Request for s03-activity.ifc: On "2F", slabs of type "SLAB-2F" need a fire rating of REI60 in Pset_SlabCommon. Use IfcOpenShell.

First a look at what the model holds.

```python
import ifcopenshell
import ifcopenshell.util.element

model = ifcopenshell.open("s03-activity.ifc")
print(model.schema)
storey = next(s for s in model.by_type("IfcBuildingStorey") if s.Name == "2F")
slabs = [e for e in ifcopenshell.util.element.get_decomposition(storey) if e.is_a("IfcSlab")]
seen = {}
for e in slabs:
    element_type = ifcopenshell.util.element.get_type(e)
    key = (element_type.Name if element_type != e and element_type else None, ifcopenshell.util.element.get_pset(e, "Pset_SlabCommon", "FireRating"))
    seen[key] = seen.get(key, 0) + 1
for (name, value), count in sorted(seen.items(), key=str):
    print(count, "x", name, "|", value)
```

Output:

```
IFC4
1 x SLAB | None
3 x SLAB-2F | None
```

```python
import ifcopenshell
import ifcopenshell.api.pset
import ifcopenshell.util.element

model = ifcopenshell.open("s03-activity.ifc")

storey = next(s for s in model.by_type("IfcBuildingStorey") if s.Name == "2F")
slabs = [e for e in ifcopenshell.util.element.get_decomposition(storey) if e.is_a("IfcSlab")]

count = 0
for e in slabs:
    element_type = ifcopenshell.util.element.get_type(e)
    if element_type in (None, e) or element_type.Name != "SLAB-2F":
        continue
    # add_pset returns the element's existing set when there is one.
    pset = ifcopenshell.api.pset.add_pset(model, product=e, name="Pset_SlabCommon")
    ifcopenshell.api.pset.edit_pset(model, pset=pset, properties={"FireRating": "REI60"})
    count += 1

print(count, "slabs updated")

model.write("s03-activity-out.ifc")
```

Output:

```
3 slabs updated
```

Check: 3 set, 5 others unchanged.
